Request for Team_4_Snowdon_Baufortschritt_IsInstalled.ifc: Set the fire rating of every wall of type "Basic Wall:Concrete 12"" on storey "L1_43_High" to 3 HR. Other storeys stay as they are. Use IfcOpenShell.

First a look at what the model holds.

```python
import ifcopenshell
import ifcopenshell.util.element

model = ifcopenshell.open("Team_4_Snowdon_Baufortschritt_IsInstalled.ifc")
print(model.schema)
storey = next(s for s in model.by_type("IfcBuildingStorey") if s.Name == "L1_43_High")
walls = [e for e in ifcopenshell.util.element.get_decomposition(storey) if e.is_a("IfcWall")]
seen = {}
for e in walls:
    element_type = ifcopenshell.util.element.get_type(e)
    key = (element_type.Name if element_type != e and element_type else None, ifcopenshell.util.element.get_pset(e, "Pset_WallCommon", "FireRating"))
    seen[key] = seen.get(key, 0) + 1
for (name, value), count in sorted(seen.items(), key=str):
    print(count, "x", name, "|", value)
```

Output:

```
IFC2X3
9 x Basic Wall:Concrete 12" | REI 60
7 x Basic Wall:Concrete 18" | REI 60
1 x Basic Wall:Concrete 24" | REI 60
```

```python
import ifcopenshell
import ifcopenshell.api.pset
import ifcopenshell.util.element

model = ifcopenshell.open("Team_4_Snowdon_Baufortschritt_IsInstalled.ifc")

storey = next(s for s in model.by_type("IfcBuildingStorey") if s.Name == "L1_43_High")
walls = [e for e in ifcopenshell.util.element.get_decomposition(storey) if e.is_a("IfcWall")]

count = 0
for e in walls:
    element_type = ifcopenshell.util.element.get_type(e)
    if element_type in (None, e) or element_type.Name != 'Basic Wall:Concrete 12"':
        continue
    # add_pset returns the element's existing set when there is one.
    pset = ifcopenshell.api.pset.add_pset(model, product=e, name="Pset_WallCommon")
    ifcopenshell.api.pset.edit_pset(model, pset=pset, properties={"FireRating": "3 HR"})
    count += 1

print(count, "walls updated")

model.write("Team_4_Snowdon_Baufortschritt_IsInstalled_edited.ifc")
```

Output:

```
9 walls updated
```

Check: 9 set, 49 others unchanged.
